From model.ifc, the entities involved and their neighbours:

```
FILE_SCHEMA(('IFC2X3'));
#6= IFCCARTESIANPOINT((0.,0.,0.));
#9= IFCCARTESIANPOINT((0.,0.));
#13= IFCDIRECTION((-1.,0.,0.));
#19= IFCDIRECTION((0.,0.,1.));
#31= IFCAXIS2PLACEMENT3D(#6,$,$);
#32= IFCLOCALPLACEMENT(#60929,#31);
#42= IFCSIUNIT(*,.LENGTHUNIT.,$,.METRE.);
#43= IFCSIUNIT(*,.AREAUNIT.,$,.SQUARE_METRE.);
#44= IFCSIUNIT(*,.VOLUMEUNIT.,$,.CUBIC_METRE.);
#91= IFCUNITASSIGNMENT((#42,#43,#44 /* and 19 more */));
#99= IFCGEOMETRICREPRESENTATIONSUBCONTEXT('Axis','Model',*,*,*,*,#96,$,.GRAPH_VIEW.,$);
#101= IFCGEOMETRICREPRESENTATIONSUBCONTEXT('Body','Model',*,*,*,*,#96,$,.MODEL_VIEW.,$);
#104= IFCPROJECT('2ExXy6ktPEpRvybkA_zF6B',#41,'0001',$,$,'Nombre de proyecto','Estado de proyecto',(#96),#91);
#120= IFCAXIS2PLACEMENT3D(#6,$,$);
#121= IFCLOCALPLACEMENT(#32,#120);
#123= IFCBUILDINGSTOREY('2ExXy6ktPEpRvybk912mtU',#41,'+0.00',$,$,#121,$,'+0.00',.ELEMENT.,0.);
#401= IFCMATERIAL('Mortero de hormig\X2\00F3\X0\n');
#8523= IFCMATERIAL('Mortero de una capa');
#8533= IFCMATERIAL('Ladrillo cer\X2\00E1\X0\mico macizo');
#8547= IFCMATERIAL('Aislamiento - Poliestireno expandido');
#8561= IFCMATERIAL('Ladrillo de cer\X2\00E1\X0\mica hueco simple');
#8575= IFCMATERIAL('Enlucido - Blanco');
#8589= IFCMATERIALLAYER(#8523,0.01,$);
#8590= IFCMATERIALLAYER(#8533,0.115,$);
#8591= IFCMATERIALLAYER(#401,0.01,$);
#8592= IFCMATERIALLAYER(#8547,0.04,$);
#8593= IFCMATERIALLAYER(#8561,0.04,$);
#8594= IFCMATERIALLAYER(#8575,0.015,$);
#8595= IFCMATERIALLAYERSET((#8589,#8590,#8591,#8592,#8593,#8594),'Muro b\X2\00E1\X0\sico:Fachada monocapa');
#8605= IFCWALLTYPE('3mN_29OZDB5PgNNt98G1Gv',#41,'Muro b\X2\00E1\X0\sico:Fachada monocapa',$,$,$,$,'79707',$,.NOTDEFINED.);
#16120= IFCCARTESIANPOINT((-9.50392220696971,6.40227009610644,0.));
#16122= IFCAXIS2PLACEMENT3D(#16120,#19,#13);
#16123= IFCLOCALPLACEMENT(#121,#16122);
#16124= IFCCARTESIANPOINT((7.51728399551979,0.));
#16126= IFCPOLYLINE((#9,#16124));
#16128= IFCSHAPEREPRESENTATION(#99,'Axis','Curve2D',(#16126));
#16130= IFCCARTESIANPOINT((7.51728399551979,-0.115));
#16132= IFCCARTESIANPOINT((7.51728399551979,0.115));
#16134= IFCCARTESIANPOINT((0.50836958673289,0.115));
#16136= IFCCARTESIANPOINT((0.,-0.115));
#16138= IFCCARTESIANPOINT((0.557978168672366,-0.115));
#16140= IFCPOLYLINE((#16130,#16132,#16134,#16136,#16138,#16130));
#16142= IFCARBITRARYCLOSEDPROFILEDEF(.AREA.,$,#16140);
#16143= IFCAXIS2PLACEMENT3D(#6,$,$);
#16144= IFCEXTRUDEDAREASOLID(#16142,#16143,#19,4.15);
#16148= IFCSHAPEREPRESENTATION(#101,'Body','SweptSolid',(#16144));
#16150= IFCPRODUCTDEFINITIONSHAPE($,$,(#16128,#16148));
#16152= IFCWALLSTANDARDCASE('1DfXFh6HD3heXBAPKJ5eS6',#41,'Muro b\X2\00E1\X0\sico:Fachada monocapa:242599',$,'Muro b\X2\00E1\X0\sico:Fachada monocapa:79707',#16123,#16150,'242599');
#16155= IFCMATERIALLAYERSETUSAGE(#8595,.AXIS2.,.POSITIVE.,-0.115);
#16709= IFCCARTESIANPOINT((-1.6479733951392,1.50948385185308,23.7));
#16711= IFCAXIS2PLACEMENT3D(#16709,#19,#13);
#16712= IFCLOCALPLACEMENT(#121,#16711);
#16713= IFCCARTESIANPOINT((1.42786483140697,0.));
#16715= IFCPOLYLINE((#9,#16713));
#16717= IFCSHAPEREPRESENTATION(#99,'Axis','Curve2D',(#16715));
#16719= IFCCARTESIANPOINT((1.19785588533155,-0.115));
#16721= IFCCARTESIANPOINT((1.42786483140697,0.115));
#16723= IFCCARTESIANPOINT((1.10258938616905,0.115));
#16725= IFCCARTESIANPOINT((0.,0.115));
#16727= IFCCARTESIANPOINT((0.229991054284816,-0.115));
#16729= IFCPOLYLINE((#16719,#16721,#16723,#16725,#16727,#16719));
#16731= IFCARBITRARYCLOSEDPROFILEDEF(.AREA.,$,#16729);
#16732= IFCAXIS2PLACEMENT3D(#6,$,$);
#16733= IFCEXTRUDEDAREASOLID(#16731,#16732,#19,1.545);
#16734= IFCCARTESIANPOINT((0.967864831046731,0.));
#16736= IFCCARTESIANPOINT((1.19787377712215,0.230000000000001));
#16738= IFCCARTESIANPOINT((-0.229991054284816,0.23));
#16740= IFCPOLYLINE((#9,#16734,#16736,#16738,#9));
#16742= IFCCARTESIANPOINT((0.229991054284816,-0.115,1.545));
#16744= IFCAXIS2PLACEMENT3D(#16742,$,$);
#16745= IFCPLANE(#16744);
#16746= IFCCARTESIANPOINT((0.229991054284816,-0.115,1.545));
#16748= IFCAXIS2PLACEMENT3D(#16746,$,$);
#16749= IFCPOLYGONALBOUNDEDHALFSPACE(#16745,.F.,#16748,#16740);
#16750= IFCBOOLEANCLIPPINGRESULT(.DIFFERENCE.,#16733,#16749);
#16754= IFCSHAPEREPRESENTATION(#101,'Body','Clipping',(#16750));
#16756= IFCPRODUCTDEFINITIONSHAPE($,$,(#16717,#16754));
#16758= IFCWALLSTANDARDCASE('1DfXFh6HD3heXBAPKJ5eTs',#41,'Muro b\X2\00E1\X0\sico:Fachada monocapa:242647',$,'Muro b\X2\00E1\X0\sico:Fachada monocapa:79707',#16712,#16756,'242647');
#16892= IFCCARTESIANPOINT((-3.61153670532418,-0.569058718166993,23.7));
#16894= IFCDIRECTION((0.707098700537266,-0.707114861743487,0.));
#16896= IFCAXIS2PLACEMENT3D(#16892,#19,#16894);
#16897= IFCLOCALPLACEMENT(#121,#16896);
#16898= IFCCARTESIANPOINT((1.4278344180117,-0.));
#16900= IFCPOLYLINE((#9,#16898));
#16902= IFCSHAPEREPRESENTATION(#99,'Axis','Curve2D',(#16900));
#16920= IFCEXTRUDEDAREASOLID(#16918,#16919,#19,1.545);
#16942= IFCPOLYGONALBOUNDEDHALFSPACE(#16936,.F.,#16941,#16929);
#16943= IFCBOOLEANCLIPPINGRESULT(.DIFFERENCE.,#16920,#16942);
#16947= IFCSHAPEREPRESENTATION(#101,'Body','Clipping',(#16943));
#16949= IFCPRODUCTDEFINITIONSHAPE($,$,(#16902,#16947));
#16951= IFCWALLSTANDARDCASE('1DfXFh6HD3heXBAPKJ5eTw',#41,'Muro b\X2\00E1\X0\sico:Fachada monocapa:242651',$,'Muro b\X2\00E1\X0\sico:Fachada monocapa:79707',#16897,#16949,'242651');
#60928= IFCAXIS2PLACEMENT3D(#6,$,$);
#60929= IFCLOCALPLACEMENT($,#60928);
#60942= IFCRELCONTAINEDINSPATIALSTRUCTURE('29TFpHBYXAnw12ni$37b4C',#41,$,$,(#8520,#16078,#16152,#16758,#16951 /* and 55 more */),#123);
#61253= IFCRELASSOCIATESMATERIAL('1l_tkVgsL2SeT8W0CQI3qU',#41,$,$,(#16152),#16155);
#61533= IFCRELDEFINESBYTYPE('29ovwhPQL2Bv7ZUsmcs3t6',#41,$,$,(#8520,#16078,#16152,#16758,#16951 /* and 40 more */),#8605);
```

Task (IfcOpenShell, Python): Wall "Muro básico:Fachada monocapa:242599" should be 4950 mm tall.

```python
import ifcopenshell
import ifcopenshell.geom
import ifcopenshell.util.representation
import ifcopenshell.util.shape
import ifcopenshell.util.unit

model = ifcopenshell.open("model.ifc")
unit_scale = ifcopenshell.util.unit.calculate_unit_scale(model)
settings = ifcopenshell.geom.settings()


def volume(element):
    """Net volume in cubic metres, openings subtracted."""
    shape = ifcopenshell.geom.create_shape(settings, element)
    return ifcopenshell.util.shape.get_volume(shape.geometry)


wall = model.by_id(16152)
before = volume(wall)

body = ifcopenshell.util.representation.get_representation(wall, "Model", "Body")
solid = body.Items[0]
old_height = solid.Depth
solid.Depth = 4.95 / unit_scale
after = volume(wall)

print(f"height {old_height:g} -> {solid.Depth:g}, volume {before:.3f} -> {after:.3f} m3")

model.write("model_updated.ifc")
```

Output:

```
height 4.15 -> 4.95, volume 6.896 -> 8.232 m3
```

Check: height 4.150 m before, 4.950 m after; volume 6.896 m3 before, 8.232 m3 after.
